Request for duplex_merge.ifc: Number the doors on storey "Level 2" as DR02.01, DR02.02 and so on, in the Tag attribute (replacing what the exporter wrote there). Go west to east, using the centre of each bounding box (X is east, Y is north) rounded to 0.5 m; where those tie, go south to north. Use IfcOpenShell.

First a look at what the model holds.

```python
import ifcopenshell
import ifcopenshell.util.element
import ifcopenshell.util.placement

model = ifcopenshell.open("duplex_merge.ifc")
print(model.schema)
storey = next(s for s in model.by_type("IfcBuildingStorey") if s.Name == "Level 2")
doors = [e for e in ifcopenshell.util.element.get_decomposition(storey) if e.is_a("IfcDoor")]
for e in sorted(doors, key=lambda e: e.id()):
    origin = ifcopenshell.util.placement.get_local_placement(e.ObjectPlacement)[:3, 3]
    print(e.id(), e.Tag, e.Name, origin.round(2) + 0.0, sep=" | ")
```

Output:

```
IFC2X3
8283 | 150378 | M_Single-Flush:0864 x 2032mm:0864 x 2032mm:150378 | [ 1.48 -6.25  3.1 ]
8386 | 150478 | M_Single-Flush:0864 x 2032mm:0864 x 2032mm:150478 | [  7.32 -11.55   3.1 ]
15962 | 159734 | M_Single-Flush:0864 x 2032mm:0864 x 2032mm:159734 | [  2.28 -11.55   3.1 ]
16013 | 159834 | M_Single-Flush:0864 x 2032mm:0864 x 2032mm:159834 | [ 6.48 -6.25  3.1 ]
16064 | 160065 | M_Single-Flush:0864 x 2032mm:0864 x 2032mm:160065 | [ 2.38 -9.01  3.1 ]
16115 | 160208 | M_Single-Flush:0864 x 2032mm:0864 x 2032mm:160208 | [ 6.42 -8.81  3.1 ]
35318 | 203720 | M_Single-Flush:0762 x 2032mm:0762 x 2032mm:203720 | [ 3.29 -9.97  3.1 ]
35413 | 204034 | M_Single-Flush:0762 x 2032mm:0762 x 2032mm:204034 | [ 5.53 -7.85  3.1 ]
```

```python
import ifcopenshell
import ifcopenshell.geom
import ifcopenshell.util.element
import ifcopenshell.util.shape

model = ifcopenshell.open("duplex_merge.ifc")
settings = ifcopenshell.geom.settings()
settings.set("use-world-coords", True)


def centre(element):
    shape = ifcopenshell.geom.create_shape(settings, element)
    return ifcopenshell.util.shape.get_bbox_centroid(shape.geometry)


storey = next(s for s in model.by_type("IfcBuildingStorey") if s.Name == "Level 2")
doors = [e for e in ifcopenshell.util.element.get_decomposition(storey) if e.is_a("IfcDoor")]

# Insertion points can sit at a corner or the storey origin, so sort by the geometry (in metres).
centres = {e: centre(e) for e in doors}
doors.sort(key=lambda e: (round(centres[e][0] / 0.5), centres[e][1]))

for i, e in enumerate(doors, start=1):
    number = f"DR02.{i:02d}"
    e.Tag = number
    print(e.id(), number)

model.write("duplex_merge-out.ifc")
```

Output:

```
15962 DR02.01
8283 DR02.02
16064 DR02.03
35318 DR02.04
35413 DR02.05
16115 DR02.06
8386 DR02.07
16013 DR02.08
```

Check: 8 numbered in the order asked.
